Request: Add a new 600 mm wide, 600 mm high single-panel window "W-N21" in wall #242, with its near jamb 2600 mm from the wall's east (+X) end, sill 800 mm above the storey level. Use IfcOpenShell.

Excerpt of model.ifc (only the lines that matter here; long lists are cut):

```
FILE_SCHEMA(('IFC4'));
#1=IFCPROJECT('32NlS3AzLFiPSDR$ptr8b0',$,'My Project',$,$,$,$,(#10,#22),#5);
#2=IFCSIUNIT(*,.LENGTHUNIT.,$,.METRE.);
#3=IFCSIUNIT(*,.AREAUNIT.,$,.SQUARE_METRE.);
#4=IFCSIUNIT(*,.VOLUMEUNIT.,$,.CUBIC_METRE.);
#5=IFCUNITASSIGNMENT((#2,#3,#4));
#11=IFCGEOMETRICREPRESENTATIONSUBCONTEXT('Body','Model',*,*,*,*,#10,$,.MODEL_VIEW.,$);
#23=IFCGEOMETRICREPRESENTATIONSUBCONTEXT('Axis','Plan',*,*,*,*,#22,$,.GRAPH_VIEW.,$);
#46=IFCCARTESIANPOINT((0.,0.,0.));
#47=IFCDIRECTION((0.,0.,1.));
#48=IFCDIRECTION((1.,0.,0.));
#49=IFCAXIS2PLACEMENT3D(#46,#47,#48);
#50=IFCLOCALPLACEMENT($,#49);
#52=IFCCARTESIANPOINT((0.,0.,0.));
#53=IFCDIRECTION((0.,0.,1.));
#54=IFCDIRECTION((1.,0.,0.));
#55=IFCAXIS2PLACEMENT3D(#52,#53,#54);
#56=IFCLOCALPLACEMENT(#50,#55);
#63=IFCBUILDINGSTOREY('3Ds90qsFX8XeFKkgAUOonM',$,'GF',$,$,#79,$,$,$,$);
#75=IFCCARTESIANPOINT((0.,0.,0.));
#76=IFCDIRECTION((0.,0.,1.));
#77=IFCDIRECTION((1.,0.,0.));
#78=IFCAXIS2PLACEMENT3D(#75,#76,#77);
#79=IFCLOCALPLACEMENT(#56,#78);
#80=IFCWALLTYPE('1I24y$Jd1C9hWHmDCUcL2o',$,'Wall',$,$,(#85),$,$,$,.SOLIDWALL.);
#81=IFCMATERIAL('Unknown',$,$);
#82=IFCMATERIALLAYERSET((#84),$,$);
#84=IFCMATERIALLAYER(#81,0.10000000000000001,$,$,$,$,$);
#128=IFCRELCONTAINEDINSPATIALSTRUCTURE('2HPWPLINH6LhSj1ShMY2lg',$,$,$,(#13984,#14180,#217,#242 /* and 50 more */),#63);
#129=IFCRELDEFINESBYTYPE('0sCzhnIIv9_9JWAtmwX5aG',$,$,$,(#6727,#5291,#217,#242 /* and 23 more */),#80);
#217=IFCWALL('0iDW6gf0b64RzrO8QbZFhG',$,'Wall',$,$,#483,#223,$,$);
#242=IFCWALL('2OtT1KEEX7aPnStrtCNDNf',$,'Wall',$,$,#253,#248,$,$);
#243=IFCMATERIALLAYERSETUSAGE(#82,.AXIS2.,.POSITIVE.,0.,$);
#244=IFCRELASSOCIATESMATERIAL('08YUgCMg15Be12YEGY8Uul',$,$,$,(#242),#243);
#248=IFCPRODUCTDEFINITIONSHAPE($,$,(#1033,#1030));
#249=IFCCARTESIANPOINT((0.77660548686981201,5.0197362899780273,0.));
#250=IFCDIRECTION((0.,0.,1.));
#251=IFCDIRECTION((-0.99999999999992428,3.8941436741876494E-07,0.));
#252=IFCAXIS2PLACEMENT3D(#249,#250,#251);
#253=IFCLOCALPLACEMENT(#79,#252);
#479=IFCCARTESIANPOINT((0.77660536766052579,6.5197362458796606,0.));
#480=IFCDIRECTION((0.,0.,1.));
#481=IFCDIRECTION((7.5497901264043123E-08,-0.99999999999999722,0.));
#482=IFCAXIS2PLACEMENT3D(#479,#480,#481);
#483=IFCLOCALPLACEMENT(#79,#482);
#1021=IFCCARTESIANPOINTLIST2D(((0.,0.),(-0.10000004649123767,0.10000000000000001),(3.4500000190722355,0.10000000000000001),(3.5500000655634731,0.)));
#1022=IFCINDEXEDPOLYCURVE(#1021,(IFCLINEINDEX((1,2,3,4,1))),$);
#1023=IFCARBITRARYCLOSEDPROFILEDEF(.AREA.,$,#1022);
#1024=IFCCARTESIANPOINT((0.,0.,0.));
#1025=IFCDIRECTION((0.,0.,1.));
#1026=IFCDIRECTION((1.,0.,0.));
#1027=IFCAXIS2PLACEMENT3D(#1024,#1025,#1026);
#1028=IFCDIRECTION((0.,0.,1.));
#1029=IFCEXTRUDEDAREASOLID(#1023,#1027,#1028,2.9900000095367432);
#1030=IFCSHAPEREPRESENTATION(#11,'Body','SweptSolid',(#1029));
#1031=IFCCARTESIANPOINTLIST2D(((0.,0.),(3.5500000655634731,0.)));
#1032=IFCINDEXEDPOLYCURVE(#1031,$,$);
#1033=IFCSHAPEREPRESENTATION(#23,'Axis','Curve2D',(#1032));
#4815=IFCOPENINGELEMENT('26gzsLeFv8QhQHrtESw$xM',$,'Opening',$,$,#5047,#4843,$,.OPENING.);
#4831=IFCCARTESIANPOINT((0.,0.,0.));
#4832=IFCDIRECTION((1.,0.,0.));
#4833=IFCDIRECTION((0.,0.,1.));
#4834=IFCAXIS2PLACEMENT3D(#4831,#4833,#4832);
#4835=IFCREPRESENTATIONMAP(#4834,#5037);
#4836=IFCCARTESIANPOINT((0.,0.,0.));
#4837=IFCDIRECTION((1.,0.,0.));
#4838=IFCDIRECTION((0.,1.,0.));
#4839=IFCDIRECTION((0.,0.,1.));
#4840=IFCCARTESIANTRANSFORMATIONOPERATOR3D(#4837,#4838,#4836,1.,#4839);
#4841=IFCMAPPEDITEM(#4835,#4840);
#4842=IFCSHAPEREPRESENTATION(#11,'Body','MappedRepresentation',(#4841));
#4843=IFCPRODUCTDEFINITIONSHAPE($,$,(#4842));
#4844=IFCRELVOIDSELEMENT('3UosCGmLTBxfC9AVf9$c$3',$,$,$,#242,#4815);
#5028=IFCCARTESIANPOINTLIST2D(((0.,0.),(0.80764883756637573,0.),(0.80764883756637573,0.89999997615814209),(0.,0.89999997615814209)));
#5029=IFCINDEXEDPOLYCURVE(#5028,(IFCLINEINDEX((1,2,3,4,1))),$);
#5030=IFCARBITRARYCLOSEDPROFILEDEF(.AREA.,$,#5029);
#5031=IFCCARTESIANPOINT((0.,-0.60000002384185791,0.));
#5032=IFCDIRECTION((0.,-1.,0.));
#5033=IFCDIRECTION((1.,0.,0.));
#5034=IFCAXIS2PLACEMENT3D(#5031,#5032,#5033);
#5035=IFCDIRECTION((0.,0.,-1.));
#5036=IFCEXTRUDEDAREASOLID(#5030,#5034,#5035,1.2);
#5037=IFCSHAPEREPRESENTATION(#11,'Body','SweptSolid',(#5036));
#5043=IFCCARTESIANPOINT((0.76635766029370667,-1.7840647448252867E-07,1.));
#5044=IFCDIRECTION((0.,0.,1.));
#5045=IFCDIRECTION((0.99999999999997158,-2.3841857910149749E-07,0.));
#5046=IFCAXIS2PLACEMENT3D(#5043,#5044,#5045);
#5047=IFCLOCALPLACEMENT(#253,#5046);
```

```python
import numpy as np
import ifcopenshell
import ifcopenshell.api.feature
import ifcopenshell.api.geometry
import ifcopenshell.api.root
import ifcopenshell.api.spatial
import ifcopenshell.geom
import ifcopenshell.util.element
import ifcopenshell.util.placement
import ifcopenshell.util.representation
import ifcopenshell.util.shape
import ifcopenshell.util.unit

model = ifcopenshell.open("model.ifc")
unit_scale = ifcopenshell.util.unit.calculate_unit_scale(model)
settings = ifcopenshell.geom.settings()


def volume(element):
    """Net volume in cubic metres, openings subtracted."""
    shape = ifcopenshell.geom.create_shape(settings, element)
    return ifcopenshell.util.shape.get_volume(shape.geometry)


wall = model.by_guid("2OtT1KEEX7aPnStrtCNDNf")
storey = ifcopenshell.util.element.get_container(wall, ifc_class="IfcBuildingStorey")
context = ifcopenshell.util.representation.get_context(model, "Model", "Body", "MODEL_VIEW")
before = volume(wall)

width, height, from_end, sill = 0.6, 0.6, 2.6, 0.8  # metres

# The wall runs along its own X axis, and the end named is its -X end.
wall_shape = ifcopenshell.geom.create_shape(settings, wall)
x, y, z = ifcopenshell.util.shape.get_vertices(wall_shape.geometry).T
start = x.min() + from_end
face, thickness = float(y.min()), float(y.max() - y.min())
wall_matrix = ifcopenshell.util.placement.get_local_placement(wall.ObjectPlacement)
level = ifcopenshell.util.placement.get_local_placement(storey.ObjectPlacement)[2, 3]


def in_wall(x, y):
    """Placement at x, y metres in the wall's axes, at sill height."""
    matrix = wall_matrix.copy()
    matrix[:, 3] = wall_matrix @ np.array([x / unit_scale, y / unit_scale, 0.0, 1.0])
    matrix[2, 3] = level + sill / unit_scale
    return matrix


# Opening: a box that overshoots both wall faces by 50 mm.
opening = ifcopenshell.api.root.create_entity(model, ifc_class="IfcOpeningElement", predefined_type="OPENING")
box = ifcopenshell.api.geometry.add_wall_representation(
    model, context=context, length=width, height=height, thickness=thickness + 0.1
)
ifcopenshell.api.geometry.assign_representation(model, product=opening, representation=box)
ifcopenshell.api.geometry.edit_object_placement(model, product=opening, matrix=in_wall(start, face - 0.05), is_si=False)
ifcopenshell.api.feature.add_feature(model, feature=opening, element=wall)

window = ifcopenshell.api.root.create_entity(model, ifc_class="IfcWindow", name="W-N21", predefined_type="WINDOW")
window.OverallWidth, window.OverallHeight = width / unit_scale, height / unit_scale
window.PartitioningType = "SINGLE_PANEL"
body = ifcopenshell.api.geometry.add_window_representation(
    model,
    context=context,
    overall_width=window.OverallWidth,
    overall_height=window.OverallHeight,
    partition_type="SINGLE_PANEL",
)
ifcopenshell.api.geometry.assign_representation(model, product=window, representation=body)
ifcopenshell.api.spatial.assign_container(model, products=[window], relating_structure=storey)
ifcopenshell.api.feature.add_filling(model, opening=opening, element=window)

# Centre the window in the wall's thickness.
ifcopenshell.api.geometry.edit_object_placement(model, product=window, matrix=in_wall(start, face), is_si=False)
window_shape = ifcopenshell.geom.create_shape(settings, window)
depth = ifcopenshell.util.shape.get_vertices(window_shape.geometry)[:, 1]
offset = face + thickness / 2 - (depth.min() + depth.max()) / 2
ifcopenshell.api.geometry.edit_object_placement(model, product=window, matrix=in_wall(start, offset), is_si=False)

after = volume(wall)

print(f"wall volume {before:.3f} -> {after:.3f} m3")

model.write("model_edited.ifc")
```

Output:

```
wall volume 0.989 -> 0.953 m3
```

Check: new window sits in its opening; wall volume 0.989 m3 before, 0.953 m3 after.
